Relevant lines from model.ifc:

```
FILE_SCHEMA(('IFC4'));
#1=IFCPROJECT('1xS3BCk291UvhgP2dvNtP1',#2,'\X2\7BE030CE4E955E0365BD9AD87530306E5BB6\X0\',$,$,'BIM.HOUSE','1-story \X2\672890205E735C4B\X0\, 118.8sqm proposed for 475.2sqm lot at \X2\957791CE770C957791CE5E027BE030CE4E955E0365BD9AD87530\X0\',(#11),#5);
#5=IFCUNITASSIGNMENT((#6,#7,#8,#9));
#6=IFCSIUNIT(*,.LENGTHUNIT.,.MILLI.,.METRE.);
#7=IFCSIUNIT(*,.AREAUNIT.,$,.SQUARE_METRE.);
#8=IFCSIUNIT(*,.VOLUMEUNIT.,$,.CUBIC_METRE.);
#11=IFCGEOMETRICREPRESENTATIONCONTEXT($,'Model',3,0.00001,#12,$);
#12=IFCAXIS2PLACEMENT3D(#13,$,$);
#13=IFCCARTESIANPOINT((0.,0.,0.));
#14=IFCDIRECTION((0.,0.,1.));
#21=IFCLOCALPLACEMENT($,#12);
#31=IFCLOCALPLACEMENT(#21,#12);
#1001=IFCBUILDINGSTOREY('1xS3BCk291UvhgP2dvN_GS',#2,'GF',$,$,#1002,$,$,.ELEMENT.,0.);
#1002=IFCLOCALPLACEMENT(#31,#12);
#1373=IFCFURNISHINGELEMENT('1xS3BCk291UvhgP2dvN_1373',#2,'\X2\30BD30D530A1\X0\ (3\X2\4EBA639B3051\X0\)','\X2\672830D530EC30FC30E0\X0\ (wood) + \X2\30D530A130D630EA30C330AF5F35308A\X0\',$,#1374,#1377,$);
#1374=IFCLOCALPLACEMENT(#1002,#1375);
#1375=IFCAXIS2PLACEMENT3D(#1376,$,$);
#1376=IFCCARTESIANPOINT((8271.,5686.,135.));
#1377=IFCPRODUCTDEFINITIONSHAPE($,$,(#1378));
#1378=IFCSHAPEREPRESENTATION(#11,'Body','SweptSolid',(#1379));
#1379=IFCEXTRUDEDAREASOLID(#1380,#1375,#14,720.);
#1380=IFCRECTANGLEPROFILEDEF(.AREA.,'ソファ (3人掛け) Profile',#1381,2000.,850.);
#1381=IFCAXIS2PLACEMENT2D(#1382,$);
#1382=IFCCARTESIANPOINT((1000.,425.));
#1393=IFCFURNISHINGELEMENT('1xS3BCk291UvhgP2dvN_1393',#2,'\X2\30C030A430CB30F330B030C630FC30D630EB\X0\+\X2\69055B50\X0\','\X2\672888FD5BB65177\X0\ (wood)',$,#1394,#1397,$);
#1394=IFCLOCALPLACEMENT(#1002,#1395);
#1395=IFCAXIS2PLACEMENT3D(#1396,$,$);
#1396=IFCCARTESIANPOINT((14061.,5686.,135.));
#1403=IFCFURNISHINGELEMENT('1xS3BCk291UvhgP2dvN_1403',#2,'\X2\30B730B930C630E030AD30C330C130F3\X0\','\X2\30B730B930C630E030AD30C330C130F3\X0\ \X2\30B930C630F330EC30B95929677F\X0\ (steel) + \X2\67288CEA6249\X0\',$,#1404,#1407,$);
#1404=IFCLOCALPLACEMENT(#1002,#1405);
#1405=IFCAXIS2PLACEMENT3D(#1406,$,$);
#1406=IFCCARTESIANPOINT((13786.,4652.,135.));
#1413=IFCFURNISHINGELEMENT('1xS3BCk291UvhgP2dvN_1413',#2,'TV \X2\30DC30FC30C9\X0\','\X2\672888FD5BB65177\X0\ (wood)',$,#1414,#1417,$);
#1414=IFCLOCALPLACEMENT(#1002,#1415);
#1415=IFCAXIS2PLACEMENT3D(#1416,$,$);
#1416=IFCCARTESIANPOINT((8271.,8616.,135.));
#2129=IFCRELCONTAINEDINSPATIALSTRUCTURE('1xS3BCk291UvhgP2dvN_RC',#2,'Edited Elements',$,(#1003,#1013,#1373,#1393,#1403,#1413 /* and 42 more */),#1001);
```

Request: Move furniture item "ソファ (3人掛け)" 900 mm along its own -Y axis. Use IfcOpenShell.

```python
import ifcopenshell
import ifcopenshell.api.geometry
import ifcopenshell.util.placement

model = ifcopenshell.open("model.ifc")

item = model.by_guid("1xS3BCk291UvhgP2dvN_1373")
matrix = ifcopenshell.util.placement.get_local_placement(item.ObjectPlacement)
matrix[:3, 3] -= matrix[:3, 1] * 900.0
ifcopenshell.api.geometry.edit_object_placement(model, product=item, matrix=matrix, is_si=False)

print(ifcopenshell.util.placement.get_local_placement(item.ObjectPlacement).round(3) + 0.0)

model.write("model_edited.ifc")
```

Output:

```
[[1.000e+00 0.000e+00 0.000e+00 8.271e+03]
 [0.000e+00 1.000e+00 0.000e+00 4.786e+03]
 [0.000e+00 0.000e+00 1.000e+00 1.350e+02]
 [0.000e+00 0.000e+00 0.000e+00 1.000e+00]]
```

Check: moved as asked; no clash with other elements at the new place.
